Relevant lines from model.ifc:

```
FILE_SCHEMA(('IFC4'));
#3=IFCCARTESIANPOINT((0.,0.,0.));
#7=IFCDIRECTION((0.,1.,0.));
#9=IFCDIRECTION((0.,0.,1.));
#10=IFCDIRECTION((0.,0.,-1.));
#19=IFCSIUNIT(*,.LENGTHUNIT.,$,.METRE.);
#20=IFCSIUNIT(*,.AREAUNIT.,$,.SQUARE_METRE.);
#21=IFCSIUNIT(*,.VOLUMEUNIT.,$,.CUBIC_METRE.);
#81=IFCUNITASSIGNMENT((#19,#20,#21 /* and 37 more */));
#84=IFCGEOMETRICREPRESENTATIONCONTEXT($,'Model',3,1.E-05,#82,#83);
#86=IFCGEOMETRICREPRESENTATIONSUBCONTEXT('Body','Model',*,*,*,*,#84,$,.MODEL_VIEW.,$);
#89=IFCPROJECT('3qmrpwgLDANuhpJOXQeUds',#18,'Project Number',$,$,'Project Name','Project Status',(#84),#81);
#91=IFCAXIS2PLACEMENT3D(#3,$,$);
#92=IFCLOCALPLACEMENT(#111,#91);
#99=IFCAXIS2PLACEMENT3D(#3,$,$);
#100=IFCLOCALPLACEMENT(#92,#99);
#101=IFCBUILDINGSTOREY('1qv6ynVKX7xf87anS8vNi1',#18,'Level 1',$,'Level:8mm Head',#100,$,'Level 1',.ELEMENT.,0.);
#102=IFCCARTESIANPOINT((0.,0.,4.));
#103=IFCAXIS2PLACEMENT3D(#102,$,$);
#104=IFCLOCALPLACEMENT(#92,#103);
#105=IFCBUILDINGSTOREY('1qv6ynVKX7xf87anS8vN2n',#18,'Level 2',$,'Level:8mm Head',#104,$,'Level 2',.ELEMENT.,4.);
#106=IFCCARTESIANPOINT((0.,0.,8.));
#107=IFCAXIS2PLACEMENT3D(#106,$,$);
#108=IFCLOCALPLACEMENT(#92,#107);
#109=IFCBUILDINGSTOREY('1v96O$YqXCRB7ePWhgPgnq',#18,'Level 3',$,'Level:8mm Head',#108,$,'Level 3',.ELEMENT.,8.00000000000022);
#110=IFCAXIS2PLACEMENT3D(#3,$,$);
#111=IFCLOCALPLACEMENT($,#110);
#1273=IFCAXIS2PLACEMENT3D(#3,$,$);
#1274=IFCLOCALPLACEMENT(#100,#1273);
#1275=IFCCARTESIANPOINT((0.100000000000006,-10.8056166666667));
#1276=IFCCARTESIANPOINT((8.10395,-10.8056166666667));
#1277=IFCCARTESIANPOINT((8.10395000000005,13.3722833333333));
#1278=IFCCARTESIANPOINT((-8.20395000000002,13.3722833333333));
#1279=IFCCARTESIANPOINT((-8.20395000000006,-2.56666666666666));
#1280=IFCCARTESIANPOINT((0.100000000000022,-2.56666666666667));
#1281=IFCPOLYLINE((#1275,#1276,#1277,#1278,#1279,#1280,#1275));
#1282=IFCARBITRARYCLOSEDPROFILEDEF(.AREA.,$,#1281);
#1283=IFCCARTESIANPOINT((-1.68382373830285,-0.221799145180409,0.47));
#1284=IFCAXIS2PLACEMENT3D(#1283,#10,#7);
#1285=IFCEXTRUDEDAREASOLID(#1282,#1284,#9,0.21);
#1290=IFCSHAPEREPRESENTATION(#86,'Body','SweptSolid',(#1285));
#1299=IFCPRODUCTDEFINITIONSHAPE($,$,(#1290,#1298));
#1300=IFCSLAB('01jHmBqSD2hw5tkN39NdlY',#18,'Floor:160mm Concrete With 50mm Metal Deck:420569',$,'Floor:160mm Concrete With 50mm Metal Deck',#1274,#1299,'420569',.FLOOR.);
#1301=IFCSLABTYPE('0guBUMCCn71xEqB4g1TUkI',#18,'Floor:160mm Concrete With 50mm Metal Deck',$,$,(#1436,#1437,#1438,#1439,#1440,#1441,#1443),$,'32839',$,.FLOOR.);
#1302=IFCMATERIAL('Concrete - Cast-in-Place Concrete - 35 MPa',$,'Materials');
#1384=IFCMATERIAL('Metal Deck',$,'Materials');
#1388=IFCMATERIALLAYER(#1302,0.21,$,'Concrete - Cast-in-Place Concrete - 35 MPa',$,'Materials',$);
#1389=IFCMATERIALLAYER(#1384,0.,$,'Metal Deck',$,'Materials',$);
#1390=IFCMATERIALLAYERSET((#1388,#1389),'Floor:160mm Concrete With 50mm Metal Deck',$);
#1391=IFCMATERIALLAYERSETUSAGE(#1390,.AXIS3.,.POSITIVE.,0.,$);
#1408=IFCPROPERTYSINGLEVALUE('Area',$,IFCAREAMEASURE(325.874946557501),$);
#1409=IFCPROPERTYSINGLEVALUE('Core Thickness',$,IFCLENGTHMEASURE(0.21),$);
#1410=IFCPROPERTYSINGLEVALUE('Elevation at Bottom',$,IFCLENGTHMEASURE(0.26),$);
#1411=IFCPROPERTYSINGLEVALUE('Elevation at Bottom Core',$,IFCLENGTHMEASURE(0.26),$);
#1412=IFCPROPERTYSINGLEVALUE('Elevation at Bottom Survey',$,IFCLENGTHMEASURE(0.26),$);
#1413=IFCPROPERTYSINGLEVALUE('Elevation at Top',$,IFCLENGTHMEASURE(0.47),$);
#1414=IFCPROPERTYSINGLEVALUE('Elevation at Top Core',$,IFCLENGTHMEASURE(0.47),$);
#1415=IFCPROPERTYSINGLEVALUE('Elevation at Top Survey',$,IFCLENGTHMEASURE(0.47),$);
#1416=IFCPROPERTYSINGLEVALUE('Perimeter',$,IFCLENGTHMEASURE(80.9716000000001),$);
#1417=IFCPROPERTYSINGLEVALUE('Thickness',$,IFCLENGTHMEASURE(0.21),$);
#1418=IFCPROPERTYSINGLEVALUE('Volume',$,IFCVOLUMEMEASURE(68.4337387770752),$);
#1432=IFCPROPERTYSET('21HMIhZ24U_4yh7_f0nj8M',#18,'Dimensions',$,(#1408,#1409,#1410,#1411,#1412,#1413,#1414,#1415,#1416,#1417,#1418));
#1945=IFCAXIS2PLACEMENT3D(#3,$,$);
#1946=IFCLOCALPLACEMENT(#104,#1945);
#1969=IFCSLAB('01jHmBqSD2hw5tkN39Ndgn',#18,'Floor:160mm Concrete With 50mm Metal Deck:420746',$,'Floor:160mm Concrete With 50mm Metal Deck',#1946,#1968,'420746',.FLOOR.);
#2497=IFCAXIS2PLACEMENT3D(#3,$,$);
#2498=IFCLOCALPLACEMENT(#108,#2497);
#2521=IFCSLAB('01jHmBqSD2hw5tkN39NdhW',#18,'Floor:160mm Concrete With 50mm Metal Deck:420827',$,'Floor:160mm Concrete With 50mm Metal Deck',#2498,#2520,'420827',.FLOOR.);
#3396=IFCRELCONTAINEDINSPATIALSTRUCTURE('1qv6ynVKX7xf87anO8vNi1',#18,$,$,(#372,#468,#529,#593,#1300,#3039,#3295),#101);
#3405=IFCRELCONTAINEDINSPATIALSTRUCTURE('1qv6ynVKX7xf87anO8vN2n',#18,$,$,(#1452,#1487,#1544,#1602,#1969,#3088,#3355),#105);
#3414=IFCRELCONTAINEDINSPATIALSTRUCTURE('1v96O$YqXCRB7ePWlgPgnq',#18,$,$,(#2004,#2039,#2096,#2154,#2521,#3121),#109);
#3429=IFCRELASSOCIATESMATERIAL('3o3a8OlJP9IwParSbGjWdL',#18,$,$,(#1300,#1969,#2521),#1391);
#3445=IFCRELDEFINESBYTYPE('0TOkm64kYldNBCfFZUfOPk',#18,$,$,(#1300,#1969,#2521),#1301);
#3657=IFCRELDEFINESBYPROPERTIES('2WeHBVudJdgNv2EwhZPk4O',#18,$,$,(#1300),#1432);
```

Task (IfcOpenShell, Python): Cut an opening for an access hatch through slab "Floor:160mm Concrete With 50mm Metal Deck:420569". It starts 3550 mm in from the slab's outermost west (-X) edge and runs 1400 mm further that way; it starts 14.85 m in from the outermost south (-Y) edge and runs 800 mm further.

```python
import numpy as np
import ifcopenshell
import ifcopenshell.api.feature
import ifcopenshell.api.geometry
import ifcopenshell.api.pset
import ifcopenshell.api.root
import ifcopenshell.geom
import ifcopenshell.util.element
import ifcopenshell.util.placement
import ifcopenshell.util.representation
import ifcopenshell.util.shape
import ifcopenshell.util.unit

model = ifcopenshell.open("model.ifc")
unit_scale = ifcopenshell.util.unit.calculate_unit_scale(model)
area_scale = ifcopenshell.util.unit.calculate_unit_scale(model, "AREAUNIT")
volume_scale = ifcopenshell.util.unit.calculate_unit_scale(model, "VOLUMEUNIT")
settings = ifcopenshell.geom.settings()


def volume(element):
    """Net volume in cubic metres, openings subtracted."""
    shape = ifcopenshell.geom.create_shape(settings, element)
    return ifcopenshell.util.shape.get_volume(shape.geometry)


slab = model.by_id(1300)
before = volume(slab)

# Extent in the slab's own axes, in metres. The edges named are its -X and -Y sides.
slab_shape = ifcopenshell.geom.create_shape(settings, slab)
vertices = ifcopenshell.util.shape.get_vertices(slab_shape.geometry)
x_min, y_min, bottom = vertices.min(axis=0)
top = vertices[:, 2].max()

opening = ifcopenshell.api.root.create_entity(model, ifc_class="IfcOpeningElement", name="Access hatch opening", predefined_type="OPENING")
context = ifcopenshell.util.representation.get_context(model, "Model", "Body", "MODEL_VIEW")
width, depth = 1.4, 0.8
outline = [(0.0, 0.0), (width, 0.0), (width, depth), (0.0, depth), (0.0, 0.0)]
# Overshoot both faces by 50 mm so the cut is clean.
shape = ifcopenshell.api.geometry.add_slab_representation(
    model, context=context, depth=top - bottom + 0.1, polyline=outline
)
ifcopenshell.api.geometry.assign_representation(model, product=opening, representation=shape)

matrix = ifcopenshell.util.placement.get_local_placement(slab.ObjectPlacement)
matrix[:, 3] = matrix @ np.append(np.array([x_min + 3.55, y_min + 14.85, bottom - 0.05]) / unit_scale, 1.0)
ifcopenshell.api.geometry.edit_object_placement(model, product=opening, matrix=matrix, is_si=False)
ifcopenshell.api.feature.add_feature(model, feature=opening, element=slab)

after = volume(slab)

# Update the slab's stored quantities.
pset = model.by_id(ifcopenshell.util.element.get_pset(slab, "Dimensions", should_inherit=False)["id"])
ifcopenshell.api.pset.edit_pset(model, pset=pset, properties={
    "Area": model.create_entity("IfcAreaMeasure", after / (top - bottom) / area_scale),
    "Volume": model.create_entity("IfcVolumeMeasure", after / volume_scale),
})

print(f"slab volume {before:.3f} -> {after:.3f} m3")

model.write("model-out.ifc")
```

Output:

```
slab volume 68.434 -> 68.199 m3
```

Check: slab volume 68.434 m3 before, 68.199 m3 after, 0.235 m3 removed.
